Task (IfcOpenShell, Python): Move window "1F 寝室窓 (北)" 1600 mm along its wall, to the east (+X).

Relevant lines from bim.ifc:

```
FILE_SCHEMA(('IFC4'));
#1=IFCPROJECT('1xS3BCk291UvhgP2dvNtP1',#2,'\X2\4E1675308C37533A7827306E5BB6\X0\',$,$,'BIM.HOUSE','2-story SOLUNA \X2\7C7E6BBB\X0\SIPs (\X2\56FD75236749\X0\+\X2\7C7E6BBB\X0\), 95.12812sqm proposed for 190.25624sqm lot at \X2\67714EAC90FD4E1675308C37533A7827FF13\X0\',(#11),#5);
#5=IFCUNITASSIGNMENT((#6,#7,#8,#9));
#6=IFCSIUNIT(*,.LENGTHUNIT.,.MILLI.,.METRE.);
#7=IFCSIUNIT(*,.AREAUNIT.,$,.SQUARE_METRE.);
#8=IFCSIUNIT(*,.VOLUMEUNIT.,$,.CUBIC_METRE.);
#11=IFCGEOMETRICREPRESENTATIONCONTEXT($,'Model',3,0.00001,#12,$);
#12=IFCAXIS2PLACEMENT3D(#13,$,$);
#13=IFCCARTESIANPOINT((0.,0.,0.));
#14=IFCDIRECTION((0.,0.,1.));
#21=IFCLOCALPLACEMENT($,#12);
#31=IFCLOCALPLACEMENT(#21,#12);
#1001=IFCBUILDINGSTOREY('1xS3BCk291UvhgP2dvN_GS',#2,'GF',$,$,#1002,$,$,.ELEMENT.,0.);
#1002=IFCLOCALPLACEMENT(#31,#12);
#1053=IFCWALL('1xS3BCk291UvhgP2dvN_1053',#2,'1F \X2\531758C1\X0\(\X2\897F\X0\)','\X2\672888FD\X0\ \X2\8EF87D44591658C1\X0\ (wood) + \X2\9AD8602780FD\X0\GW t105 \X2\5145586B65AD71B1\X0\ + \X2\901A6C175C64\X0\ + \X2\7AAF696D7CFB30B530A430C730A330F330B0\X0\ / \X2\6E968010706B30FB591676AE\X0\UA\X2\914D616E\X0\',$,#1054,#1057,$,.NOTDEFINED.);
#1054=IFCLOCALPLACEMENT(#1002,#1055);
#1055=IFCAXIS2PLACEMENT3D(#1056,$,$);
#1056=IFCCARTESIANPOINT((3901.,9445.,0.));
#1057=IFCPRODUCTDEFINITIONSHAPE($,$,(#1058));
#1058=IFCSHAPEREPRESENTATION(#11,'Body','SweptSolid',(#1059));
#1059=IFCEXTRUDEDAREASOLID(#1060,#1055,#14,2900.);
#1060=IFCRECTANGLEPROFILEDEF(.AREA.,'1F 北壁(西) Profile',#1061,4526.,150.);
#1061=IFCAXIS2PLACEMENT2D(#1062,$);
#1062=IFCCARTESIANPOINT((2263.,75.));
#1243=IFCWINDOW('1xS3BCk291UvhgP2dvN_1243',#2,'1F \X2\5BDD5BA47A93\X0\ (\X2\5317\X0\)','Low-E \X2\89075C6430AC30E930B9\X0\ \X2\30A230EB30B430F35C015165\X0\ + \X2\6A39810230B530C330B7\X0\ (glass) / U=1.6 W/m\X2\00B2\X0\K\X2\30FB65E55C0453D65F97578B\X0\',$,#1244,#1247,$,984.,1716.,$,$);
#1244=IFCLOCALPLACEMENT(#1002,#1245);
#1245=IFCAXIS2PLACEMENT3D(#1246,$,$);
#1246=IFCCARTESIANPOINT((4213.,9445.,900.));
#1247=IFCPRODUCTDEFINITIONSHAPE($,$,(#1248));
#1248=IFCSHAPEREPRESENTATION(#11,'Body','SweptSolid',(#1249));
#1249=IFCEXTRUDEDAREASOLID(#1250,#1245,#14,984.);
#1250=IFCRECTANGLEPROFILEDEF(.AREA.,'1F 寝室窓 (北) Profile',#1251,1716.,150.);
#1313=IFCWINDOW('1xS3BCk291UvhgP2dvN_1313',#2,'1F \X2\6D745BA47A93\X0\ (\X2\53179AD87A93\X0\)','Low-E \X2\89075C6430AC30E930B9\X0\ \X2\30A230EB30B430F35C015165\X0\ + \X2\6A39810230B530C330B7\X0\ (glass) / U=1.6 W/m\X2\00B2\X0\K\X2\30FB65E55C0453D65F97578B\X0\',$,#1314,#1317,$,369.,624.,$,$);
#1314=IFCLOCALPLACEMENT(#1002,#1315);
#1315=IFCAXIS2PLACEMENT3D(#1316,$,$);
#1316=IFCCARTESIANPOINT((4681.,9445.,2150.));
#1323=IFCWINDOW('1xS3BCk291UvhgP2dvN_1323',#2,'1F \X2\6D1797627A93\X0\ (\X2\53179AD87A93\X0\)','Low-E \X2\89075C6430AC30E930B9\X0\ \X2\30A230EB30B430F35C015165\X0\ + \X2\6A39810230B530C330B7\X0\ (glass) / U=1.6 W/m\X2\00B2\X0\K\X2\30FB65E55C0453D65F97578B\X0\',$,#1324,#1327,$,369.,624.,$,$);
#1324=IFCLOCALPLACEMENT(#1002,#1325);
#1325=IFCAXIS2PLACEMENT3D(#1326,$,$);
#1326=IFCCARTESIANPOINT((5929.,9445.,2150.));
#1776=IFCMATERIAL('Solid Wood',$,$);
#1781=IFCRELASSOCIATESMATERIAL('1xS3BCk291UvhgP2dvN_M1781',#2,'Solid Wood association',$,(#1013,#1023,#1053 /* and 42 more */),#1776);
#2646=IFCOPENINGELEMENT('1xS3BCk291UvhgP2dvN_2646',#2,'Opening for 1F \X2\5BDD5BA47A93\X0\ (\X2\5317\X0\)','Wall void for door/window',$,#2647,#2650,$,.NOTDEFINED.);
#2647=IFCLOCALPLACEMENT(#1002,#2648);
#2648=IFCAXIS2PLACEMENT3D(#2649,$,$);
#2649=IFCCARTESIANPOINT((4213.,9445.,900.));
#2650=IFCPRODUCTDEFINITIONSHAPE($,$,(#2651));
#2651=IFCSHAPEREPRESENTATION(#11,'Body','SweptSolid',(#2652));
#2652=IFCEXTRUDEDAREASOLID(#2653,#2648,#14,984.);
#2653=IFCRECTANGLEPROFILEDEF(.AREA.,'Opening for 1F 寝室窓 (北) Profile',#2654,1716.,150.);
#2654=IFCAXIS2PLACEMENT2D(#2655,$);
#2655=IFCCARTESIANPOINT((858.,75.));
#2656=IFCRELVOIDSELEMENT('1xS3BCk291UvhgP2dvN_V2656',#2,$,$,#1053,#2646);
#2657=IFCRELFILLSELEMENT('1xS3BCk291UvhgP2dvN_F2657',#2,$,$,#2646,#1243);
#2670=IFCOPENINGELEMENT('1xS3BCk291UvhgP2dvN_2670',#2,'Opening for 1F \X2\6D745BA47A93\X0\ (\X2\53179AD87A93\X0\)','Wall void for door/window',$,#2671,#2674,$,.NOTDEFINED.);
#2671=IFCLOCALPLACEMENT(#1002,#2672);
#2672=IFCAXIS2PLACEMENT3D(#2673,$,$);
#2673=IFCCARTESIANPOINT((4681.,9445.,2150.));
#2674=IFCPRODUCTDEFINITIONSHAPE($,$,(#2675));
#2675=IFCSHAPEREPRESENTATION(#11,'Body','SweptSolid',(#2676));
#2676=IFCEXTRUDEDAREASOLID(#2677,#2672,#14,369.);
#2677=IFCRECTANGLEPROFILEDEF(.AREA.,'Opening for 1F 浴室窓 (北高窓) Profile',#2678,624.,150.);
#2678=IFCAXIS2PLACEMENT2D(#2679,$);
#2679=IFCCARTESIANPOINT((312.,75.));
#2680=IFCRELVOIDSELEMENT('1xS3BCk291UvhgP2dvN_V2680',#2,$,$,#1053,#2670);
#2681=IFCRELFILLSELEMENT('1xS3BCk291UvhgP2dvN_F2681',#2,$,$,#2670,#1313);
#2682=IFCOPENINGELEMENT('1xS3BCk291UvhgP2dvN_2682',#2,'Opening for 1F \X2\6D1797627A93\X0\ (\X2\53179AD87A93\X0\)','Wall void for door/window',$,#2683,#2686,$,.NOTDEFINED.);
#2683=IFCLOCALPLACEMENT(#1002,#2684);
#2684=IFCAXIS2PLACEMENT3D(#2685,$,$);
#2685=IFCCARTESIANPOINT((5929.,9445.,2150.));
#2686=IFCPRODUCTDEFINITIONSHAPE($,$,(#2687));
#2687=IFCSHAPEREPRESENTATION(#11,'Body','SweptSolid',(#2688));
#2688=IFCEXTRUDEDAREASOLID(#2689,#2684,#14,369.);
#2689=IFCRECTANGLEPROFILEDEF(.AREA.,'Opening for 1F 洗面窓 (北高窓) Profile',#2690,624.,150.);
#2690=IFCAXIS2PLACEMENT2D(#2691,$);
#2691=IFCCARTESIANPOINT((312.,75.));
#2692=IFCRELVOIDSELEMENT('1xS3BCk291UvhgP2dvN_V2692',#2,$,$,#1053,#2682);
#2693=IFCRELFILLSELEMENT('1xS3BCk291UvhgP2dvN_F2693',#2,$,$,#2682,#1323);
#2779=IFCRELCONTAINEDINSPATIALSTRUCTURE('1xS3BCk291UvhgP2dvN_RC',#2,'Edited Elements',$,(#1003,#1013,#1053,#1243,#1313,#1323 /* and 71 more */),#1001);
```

```python
import ifcopenshell
import ifcopenshell.api.geometry
import ifcopenshell.util.placement

model = ifcopenshell.open("bim.ifc")

window = model.by_guid("1xS3BCk291UvhgP2dvN_1243")
opening = window.FillsVoids[0].RelatingOpeningElement
wall = opening.VoidsElements[0].RelatingBuildingElement

wall_matrix = ifcopenshell.util.placement.get_local_placement(wall.ObjectPlacement)
shift = wall_matrix[:3, 0] * 1600.0
before = ifcopenshell.util.placement.get_local_placement(window.ObjectPlacement)[:3, 3].copy()

# The window is not placed relative to its opening, so move both.
for product in (opening, window):
    matrix = ifcopenshell.util.placement.get_local_placement(product.ObjectPlacement)
    matrix[:3, 3] += shift
    ifcopenshell.api.geometry.edit_object_placement(model, product=product, matrix=matrix, is_si=False)

after = ifcopenshell.util.placement.get_local_placement(window.ObjectPlacement)[:3, 3]
print("window moved by", (after - before).round(3) + 0.0)

model.write("bim_v2.ifc")
```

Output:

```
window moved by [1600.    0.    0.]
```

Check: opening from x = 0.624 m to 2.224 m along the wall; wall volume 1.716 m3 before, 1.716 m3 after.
